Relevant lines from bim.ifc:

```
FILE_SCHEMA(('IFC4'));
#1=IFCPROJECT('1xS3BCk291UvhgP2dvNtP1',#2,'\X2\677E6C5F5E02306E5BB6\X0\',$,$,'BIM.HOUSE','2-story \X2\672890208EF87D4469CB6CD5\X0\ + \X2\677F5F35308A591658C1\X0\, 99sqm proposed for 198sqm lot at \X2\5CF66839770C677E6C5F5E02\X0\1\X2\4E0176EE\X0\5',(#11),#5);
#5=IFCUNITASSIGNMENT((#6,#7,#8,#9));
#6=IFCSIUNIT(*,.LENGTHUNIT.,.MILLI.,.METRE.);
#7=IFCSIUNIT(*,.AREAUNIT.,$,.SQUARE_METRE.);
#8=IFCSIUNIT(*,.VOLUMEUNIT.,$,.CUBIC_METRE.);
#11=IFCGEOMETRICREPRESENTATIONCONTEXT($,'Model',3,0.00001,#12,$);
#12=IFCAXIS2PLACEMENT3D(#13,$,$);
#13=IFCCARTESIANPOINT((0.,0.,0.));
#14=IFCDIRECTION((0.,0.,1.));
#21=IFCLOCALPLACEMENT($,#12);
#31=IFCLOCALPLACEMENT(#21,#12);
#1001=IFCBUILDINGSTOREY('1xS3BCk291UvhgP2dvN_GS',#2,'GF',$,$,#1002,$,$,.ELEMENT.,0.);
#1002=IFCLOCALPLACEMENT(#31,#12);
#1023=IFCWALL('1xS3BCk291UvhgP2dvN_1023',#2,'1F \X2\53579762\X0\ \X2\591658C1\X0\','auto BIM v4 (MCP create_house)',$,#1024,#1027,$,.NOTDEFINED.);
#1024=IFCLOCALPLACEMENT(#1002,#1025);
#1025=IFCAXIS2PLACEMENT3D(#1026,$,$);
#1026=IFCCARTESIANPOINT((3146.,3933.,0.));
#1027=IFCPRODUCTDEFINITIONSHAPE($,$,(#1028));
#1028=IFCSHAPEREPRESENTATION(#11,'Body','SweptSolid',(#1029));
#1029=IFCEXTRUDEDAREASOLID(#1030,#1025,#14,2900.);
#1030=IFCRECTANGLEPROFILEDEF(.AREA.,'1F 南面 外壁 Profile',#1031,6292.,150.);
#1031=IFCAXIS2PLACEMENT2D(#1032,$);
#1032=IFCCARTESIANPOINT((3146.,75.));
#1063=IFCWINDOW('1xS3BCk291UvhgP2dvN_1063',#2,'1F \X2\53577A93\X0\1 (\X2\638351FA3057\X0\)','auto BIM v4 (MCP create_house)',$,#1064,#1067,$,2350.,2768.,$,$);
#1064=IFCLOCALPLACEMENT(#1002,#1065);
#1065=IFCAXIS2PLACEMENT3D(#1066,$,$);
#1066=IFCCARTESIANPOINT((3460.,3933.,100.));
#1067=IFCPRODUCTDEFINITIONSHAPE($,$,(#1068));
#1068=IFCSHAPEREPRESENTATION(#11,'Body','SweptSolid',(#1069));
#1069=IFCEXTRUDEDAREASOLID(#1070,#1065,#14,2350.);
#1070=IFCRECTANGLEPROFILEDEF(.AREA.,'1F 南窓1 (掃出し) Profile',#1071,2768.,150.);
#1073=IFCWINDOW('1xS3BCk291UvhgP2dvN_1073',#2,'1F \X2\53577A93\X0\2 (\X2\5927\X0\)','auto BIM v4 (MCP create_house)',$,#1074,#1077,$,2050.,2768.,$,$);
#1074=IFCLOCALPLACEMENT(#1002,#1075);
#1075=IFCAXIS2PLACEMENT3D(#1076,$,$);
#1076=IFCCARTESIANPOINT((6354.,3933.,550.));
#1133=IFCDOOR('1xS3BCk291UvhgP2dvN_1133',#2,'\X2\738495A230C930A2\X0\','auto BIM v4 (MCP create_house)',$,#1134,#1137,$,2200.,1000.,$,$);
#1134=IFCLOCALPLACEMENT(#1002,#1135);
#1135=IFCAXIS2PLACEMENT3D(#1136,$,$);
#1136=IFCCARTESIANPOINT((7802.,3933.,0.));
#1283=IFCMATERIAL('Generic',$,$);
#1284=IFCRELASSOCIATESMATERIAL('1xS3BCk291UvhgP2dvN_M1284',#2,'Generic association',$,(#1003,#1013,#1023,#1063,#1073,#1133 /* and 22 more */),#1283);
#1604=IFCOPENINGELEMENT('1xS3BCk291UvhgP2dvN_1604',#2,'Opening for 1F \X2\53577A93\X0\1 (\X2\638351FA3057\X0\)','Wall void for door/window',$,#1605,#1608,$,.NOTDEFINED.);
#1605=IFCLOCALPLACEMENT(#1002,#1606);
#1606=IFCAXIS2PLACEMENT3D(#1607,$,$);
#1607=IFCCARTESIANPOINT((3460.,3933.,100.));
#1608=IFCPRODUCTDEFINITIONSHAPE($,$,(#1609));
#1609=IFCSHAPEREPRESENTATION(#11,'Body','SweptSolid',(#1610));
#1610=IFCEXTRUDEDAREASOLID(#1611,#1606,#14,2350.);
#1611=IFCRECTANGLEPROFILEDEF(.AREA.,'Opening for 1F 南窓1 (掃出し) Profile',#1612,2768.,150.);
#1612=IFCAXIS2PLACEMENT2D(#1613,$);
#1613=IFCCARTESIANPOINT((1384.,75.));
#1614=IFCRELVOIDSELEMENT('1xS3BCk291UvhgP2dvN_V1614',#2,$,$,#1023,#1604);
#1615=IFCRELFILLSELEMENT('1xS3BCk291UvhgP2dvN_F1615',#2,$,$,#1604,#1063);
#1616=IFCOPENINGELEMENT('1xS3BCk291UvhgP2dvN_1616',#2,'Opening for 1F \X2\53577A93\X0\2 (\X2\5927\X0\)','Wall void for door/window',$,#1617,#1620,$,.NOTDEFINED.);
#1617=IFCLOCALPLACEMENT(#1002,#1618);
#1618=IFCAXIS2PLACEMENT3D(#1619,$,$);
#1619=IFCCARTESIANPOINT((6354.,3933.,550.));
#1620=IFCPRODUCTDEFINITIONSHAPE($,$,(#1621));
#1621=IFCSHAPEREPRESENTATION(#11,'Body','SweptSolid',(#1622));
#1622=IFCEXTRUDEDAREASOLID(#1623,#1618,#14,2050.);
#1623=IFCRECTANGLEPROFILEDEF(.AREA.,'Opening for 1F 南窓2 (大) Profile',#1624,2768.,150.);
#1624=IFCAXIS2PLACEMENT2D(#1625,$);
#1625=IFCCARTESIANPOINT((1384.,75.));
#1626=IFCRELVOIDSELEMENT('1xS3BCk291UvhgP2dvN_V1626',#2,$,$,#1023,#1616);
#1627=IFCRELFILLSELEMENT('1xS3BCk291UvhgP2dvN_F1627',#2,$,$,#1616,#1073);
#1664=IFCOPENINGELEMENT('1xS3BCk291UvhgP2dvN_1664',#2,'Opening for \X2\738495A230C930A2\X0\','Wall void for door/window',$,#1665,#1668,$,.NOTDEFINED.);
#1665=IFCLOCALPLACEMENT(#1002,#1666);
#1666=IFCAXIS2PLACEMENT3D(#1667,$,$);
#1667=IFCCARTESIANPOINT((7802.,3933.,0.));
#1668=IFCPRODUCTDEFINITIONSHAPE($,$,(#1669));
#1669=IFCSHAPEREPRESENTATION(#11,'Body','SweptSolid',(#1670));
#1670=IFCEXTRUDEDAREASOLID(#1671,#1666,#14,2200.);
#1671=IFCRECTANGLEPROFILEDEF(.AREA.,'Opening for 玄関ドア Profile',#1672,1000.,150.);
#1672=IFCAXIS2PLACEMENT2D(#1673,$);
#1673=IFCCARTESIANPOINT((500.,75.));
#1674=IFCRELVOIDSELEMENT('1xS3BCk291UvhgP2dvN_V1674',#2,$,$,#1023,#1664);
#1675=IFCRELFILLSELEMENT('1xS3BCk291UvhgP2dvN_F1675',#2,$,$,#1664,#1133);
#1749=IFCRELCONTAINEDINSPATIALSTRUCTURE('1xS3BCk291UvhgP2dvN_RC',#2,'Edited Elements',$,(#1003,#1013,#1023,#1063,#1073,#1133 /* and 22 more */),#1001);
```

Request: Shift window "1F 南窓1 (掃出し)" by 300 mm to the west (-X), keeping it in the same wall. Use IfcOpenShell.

```python
import ifcopenshell
import ifcopenshell.api.geometry
import ifcopenshell.util.placement

model = ifcopenshell.open("bim.ifc")

window = model.by_guid("1xS3BCk291UvhgP2dvN_1063")
opening = window.FillsVoids[0].RelatingOpeningElement
wall = opening.VoidsElements[0].RelatingBuildingElement

wall_matrix = ifcopenshell.util.placement.get_local_placement(wall.ObjectPlacement)
shift = wall_matrix[:3, 0] * -300.0
before = ifcopenshell.util.placement.get_local_placement(window.ObjectPlacement)[:3, 3].copy()

# The window is not placed relative to its opening, so move both.
for product in (opening, window):
    matrix = ifcopenshell.util.placement.get_local_placement(product.ObjectPlacement)
    matrix[:3, 3] += shift
    ifcopenshell.api.geometry.edit_object_placement(model, product=product, matrix=matrix, is_si=False)

after = ifcopenshell.util.placement.get_local_placement(window.ObjectPlacement)[:3, 3]
print("window moved by", (after - before).round(3) + 0.0)

model.write("bim_updated.ifc")
```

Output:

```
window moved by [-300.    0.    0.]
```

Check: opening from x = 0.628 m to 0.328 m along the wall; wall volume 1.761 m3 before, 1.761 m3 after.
